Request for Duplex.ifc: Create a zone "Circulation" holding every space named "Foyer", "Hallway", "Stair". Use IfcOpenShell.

First a look at what the model holds.

```python
import ifcopenshell

model = ifcopenshell.open("Duplex.ifc")
print(model.schema)
seen = {}
for space in model.by_type("IfcSpace"):
    seen[space.LongName] = seen.get(space.LongName, 0) + 1
for name, count in sorted(seen.items(), key=str):
    print(count, "x", name)
print("zones:", [z.Name for z in model.by_type("IfcZone")][:20])
```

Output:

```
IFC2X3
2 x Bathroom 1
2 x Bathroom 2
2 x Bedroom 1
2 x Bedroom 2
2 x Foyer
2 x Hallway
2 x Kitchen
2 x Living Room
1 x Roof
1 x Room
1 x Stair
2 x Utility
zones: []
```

```python
import ifcopenshell
import ifcopenshell.api.group
import ifcopenshell.api.root

model = ifcopenshell.open("Duplex.ifc")

names = {"Foyer", "Hallway", "Stair"}
spaces = [s for s in model.by_type("IfcSpace") if s.LongName in names]

zone = ifcopenshell.api.root.create_entity(model, ifc_class="IfcZone", name="Circulation")
ifcopenshell.api.group.assign_group(model, products=spaces, group=zone)
print(len(spaces), "spaces in", zone.Name)

model.write("Duplex-out.ifc")
```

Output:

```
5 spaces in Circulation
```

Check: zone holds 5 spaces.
